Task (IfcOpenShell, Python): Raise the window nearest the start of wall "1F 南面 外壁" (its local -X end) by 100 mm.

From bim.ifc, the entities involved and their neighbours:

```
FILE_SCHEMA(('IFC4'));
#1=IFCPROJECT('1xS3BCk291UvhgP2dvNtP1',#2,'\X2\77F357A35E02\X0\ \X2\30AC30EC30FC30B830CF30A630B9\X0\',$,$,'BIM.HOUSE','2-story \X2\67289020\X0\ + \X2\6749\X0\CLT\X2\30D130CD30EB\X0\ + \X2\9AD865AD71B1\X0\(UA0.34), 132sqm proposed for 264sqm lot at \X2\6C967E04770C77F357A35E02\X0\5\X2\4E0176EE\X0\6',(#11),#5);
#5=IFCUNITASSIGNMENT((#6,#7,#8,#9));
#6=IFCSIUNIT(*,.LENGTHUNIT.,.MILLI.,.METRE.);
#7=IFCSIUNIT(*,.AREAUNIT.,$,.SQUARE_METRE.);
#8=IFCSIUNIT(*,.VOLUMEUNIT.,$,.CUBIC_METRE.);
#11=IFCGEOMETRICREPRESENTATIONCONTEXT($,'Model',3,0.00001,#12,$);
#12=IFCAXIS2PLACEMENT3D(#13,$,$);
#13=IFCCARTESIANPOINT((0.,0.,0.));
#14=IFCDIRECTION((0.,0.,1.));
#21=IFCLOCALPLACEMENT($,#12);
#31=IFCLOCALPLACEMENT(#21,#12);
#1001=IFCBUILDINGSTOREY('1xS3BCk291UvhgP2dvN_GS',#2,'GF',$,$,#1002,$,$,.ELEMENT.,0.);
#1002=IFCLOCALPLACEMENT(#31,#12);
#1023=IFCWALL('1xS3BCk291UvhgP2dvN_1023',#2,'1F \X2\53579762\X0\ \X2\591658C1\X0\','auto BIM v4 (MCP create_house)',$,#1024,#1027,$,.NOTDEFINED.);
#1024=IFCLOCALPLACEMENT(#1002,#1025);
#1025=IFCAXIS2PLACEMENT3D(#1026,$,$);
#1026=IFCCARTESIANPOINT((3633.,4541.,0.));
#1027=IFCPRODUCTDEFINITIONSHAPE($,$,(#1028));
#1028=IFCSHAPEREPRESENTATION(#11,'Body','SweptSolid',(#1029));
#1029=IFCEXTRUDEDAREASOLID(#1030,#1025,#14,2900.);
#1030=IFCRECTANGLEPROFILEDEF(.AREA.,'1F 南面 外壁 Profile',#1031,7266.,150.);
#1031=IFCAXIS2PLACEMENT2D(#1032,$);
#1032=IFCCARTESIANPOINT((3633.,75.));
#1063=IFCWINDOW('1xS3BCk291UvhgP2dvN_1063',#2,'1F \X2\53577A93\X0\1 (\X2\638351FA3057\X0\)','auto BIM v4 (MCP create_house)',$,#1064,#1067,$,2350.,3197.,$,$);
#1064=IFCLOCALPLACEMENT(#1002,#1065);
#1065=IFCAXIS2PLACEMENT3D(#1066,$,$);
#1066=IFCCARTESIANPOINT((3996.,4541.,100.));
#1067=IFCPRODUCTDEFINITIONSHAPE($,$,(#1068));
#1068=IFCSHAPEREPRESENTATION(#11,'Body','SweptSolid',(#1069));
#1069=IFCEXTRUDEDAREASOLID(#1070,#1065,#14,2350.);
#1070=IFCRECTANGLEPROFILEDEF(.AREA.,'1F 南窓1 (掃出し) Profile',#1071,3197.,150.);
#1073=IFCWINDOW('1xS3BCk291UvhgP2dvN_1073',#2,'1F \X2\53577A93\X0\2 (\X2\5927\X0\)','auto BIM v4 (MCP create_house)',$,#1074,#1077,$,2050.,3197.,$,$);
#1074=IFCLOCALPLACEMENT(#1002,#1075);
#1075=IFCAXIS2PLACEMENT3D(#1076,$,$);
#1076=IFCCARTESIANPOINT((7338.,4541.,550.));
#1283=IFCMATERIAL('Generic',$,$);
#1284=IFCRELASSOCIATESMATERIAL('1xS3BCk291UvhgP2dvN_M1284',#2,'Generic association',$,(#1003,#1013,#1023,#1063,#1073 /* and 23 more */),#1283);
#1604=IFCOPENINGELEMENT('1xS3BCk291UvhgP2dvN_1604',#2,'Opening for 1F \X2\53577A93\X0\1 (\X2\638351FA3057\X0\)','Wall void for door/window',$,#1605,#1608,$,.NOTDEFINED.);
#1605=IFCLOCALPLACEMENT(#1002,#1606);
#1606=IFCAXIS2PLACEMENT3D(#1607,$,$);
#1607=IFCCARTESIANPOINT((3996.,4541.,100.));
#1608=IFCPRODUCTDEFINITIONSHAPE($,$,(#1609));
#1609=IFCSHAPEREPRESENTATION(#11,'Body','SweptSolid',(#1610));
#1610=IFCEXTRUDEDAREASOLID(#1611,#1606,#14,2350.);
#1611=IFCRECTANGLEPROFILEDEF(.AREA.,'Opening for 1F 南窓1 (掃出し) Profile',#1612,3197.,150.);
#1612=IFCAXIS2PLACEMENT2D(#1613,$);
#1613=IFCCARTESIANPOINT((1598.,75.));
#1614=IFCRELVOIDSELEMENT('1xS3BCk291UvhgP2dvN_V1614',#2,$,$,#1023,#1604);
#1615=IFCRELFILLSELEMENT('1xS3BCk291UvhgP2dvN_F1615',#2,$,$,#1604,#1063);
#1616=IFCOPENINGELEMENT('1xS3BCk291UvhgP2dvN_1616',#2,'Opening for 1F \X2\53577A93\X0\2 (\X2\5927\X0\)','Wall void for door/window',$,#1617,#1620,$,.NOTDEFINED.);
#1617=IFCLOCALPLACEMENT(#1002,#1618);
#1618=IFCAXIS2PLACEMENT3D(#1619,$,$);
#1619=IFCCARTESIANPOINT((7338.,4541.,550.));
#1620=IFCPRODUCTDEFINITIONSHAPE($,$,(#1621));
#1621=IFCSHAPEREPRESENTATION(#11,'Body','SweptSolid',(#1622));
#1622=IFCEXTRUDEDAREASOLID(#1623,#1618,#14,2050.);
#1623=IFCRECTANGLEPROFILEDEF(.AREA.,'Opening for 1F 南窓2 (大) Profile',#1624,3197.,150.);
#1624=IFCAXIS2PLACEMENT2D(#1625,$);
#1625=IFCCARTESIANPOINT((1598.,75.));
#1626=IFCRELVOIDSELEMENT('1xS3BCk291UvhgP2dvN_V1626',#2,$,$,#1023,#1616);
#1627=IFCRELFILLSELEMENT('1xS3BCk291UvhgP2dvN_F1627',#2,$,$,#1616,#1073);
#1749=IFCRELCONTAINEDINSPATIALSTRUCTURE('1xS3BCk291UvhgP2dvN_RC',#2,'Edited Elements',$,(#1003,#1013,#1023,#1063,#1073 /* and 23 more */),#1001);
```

```python
import numpy as np
import ifcopenshell
import ifcopenshell.api.geometry
import ifcopenshell.util.placement
import ifcopenshell.util.unit

model = ifcopenshell.open("bim.ifc")
unit_scale = ifcopenshell.util.unit.calculate_unit_scale(model)

window = model.by_guid("1xS3BCk291UvhgP2dvN_1063")
opening = window.FillsVoids[0].RelatingOpeningElement
dz = 0.1 / unit_scale

shift = np.array([0.0, 0.0, dz])
# The window is not placed relative to its opening, so move both.
for product in (opening, window):
    matrix = ifcopenshell.util.placement.get_local_placement(product.ObjectPlacement)
    matrix[:3, 3] += shift
    ifcopenshell.api.geometry.edit_object_placement(model, product=product, matrix=matrix, is_si=False)

print(f"moved by {dz * unit_scale:+.3f} m")

model.write("bim-out.ifc")
```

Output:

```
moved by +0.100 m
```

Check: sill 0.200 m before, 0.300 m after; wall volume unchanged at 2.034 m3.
